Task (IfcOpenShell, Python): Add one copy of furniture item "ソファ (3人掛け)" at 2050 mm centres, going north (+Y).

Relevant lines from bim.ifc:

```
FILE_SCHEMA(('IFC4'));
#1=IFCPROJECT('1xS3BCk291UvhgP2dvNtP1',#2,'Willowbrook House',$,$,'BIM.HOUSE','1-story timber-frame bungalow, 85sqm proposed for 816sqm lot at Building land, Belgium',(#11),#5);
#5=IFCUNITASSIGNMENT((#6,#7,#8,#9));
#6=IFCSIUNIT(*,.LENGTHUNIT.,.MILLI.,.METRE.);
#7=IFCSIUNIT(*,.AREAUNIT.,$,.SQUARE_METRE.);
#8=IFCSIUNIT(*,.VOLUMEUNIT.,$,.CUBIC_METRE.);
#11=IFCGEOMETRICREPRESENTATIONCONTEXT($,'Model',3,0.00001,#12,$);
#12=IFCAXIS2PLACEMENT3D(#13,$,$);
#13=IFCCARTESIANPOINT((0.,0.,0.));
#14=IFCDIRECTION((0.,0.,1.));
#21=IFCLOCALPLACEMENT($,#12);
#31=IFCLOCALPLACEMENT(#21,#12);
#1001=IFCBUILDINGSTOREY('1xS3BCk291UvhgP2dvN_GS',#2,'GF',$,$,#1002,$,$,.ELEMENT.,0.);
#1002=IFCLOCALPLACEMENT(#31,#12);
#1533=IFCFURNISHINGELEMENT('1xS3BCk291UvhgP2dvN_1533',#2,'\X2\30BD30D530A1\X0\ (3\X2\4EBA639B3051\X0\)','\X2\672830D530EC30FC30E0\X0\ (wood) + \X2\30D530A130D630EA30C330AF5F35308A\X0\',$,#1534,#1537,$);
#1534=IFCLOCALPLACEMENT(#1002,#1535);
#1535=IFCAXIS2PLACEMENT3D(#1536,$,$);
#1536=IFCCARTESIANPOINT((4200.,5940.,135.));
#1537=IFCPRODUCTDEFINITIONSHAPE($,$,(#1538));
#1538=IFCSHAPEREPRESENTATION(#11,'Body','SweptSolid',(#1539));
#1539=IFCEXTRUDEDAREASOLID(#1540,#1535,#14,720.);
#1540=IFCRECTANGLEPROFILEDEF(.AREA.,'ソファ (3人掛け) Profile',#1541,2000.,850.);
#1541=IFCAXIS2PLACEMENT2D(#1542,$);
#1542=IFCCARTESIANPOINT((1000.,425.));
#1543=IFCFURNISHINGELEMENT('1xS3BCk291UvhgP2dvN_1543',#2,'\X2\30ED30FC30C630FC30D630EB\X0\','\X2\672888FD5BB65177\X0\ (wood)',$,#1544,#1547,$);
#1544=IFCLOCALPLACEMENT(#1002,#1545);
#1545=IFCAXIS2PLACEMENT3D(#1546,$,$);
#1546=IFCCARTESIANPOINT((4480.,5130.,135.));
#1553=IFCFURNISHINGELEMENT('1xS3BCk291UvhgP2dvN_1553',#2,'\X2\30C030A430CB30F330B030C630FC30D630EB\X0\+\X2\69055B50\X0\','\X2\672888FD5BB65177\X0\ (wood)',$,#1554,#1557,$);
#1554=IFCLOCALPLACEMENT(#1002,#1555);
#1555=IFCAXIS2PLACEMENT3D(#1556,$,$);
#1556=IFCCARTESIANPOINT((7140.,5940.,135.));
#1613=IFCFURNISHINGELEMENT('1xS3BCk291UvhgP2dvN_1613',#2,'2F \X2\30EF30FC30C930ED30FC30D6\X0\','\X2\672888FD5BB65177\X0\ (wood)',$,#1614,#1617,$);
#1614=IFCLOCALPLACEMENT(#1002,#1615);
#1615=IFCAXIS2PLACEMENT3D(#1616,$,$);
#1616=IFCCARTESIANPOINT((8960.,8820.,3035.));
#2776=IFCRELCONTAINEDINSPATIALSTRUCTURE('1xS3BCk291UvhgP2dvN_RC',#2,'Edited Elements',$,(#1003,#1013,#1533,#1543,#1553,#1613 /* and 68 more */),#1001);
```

```python
import numpy as np
import ifcopenshell
import ifcopenshell.api.geometry
import ifcopenshell.api.root
import ifcopenshell.util.element
import ifcopenshell.util.placement
import ifcopenshell.util.unit

model = ifcopenshell.open("bim.ifc")
unit_scale = ifcopenshell.util.unit.calculate_unit_scale(model)


def reuse_history(source, copy):
    """copy_class also copies each property set's owner history, people and application; keep the originals."""
    for rel in copy.IsDefinedBy:
        if rel.is_a("IfcRelDefinesByProperties") and (history := rel.RelatingPropertyDefinition.OwnerHistory):
            rel.RelatingPropertyDefinition.OwnerHistory = source.OwnerHistory
            ifcopenshell.util.element.remove_deep2(model, history)


source = model.by_id(1533)
base = ifcopenshell.util.placement.get_local_placement(source.ObjectPlacement)
step = np.array([0.0, 1.0, 0.0]) * 2.05 / unit_scale

for i in range(1, 2):
    copy = ifcopenshell.api.root.copy_class(model, product=source)
    copy.Representation = ifcopenshell.util.element.copy_deep(
        model, source.Representation, exclude=["IfcGeometricRepresentationContext", "IfcRepresentationMap"]
    )
    reuse_history(source, copy)
    matrix = base.copy()
    matrix[:3, 3] += i * step
    print("added at", matrix[:3, 3].round(3) + 0.0)
    ifcopenshell.api.geometry.edit_object_placement(model, product=copy, matrix=matrix, is_si=False)

model.write("bim_rev.ifc")
```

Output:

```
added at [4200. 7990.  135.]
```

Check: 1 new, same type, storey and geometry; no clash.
